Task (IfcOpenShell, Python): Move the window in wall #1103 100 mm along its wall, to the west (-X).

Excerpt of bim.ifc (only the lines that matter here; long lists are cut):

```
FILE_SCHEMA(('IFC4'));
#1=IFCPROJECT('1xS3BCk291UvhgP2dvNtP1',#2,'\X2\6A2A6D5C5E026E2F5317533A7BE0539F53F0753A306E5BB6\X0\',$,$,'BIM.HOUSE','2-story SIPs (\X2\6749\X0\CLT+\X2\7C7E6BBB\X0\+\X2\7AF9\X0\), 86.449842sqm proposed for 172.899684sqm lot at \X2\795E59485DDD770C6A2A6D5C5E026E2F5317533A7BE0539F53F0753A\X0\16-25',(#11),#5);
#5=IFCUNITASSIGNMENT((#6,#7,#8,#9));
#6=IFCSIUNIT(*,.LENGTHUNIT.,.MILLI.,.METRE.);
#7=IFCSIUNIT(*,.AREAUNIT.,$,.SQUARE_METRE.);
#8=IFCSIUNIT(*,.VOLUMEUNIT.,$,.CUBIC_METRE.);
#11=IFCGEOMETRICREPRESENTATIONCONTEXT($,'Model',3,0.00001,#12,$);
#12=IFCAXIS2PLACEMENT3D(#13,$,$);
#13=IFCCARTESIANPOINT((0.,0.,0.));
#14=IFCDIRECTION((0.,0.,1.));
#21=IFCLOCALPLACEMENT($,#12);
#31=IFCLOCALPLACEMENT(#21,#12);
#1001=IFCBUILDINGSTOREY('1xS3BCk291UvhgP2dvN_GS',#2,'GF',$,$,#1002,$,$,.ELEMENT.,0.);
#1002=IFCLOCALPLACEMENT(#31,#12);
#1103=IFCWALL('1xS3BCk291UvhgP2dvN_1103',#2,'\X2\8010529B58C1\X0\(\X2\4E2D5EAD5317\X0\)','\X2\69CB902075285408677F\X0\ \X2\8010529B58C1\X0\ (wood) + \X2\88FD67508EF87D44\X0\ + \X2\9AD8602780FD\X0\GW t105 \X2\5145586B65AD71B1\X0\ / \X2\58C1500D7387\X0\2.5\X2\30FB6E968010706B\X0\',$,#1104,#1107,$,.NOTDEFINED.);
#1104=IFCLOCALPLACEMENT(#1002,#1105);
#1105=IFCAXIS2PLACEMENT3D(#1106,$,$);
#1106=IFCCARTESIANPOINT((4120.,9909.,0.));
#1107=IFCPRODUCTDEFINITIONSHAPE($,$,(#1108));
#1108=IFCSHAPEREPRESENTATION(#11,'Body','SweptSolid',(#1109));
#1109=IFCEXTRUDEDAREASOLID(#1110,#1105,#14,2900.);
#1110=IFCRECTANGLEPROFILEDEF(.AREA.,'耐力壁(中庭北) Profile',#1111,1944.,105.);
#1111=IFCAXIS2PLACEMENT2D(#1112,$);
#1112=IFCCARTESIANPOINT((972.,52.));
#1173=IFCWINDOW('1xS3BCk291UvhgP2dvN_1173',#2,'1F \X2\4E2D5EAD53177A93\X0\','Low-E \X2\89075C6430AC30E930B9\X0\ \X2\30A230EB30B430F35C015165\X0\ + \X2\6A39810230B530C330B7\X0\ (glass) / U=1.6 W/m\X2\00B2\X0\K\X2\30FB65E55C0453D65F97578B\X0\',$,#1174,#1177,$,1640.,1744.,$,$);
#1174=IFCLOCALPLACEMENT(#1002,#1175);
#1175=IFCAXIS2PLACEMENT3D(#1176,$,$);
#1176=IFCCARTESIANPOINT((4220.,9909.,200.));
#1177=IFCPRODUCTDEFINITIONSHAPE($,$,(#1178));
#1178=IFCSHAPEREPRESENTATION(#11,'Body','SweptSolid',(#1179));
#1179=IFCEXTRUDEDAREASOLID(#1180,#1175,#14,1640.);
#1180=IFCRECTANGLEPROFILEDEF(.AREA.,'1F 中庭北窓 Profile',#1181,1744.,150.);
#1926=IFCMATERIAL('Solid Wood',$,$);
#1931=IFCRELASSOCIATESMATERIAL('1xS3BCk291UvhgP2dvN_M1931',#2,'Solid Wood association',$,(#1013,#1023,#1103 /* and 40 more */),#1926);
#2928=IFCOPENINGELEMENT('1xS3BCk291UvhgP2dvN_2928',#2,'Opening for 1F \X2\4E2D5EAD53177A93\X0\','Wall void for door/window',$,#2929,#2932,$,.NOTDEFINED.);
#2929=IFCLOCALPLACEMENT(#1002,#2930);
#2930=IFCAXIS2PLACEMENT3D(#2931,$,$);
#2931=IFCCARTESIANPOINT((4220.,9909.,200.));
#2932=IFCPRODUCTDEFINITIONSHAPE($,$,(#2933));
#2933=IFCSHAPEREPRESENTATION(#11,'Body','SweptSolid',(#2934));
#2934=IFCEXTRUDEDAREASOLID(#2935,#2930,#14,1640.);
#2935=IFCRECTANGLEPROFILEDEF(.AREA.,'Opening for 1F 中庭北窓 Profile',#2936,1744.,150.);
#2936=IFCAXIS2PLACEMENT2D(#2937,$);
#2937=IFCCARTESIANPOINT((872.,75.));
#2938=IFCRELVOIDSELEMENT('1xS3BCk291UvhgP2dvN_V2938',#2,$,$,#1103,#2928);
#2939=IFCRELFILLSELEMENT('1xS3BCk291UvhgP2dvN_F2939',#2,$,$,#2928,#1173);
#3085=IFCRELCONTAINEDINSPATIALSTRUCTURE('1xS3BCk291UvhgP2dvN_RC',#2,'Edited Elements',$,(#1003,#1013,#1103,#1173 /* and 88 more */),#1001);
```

```python
import ifcopenshell
import ifcopenshell.api.geometry
import ifcopenshell.util.placement
import ifcopenshell.util.unit

model = ifcopenshell.open("bim.ifc")
unit_scale = ifcopenshell.util.unit.calculate_unit_scale(model)

window = model.by_id(1173)
opening = window.FillsVoids[0].RelatingOpeningElement
wall = opening.VoidsElements[0].RelatingBuildingElement

wall_matrix = ifcopenshell.util.placement.get_local_placement(wall.ObjectPlacement)
shift = wall_matrix[:3, 0] * -0.1 / unit_scale
before = ifcopenshell.util.placement.get_local_placement(window.ObjectPlacement)[:3, 3].copy()

# The window is not placed relative to its opening, so move both.
for product in (opening, window):
    matrix = ifcopenshell.util.placement.get_local_placement(product.ObjectPlacement)
    matrix[:3, 3] += shift
    ifcopenshell.api.geometry.edit_object_placement(model, product=product, matrix=matrix, is_si=False)

after = ifcopenshell.util.placement.get_local_placement(window.ObjectPlacement)[:3, 3]
print("window moved by", (after - before).round(3) + 0.0)

model.write("bim_edited.ifc")
```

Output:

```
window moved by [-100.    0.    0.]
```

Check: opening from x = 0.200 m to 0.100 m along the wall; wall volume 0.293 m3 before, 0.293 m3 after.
